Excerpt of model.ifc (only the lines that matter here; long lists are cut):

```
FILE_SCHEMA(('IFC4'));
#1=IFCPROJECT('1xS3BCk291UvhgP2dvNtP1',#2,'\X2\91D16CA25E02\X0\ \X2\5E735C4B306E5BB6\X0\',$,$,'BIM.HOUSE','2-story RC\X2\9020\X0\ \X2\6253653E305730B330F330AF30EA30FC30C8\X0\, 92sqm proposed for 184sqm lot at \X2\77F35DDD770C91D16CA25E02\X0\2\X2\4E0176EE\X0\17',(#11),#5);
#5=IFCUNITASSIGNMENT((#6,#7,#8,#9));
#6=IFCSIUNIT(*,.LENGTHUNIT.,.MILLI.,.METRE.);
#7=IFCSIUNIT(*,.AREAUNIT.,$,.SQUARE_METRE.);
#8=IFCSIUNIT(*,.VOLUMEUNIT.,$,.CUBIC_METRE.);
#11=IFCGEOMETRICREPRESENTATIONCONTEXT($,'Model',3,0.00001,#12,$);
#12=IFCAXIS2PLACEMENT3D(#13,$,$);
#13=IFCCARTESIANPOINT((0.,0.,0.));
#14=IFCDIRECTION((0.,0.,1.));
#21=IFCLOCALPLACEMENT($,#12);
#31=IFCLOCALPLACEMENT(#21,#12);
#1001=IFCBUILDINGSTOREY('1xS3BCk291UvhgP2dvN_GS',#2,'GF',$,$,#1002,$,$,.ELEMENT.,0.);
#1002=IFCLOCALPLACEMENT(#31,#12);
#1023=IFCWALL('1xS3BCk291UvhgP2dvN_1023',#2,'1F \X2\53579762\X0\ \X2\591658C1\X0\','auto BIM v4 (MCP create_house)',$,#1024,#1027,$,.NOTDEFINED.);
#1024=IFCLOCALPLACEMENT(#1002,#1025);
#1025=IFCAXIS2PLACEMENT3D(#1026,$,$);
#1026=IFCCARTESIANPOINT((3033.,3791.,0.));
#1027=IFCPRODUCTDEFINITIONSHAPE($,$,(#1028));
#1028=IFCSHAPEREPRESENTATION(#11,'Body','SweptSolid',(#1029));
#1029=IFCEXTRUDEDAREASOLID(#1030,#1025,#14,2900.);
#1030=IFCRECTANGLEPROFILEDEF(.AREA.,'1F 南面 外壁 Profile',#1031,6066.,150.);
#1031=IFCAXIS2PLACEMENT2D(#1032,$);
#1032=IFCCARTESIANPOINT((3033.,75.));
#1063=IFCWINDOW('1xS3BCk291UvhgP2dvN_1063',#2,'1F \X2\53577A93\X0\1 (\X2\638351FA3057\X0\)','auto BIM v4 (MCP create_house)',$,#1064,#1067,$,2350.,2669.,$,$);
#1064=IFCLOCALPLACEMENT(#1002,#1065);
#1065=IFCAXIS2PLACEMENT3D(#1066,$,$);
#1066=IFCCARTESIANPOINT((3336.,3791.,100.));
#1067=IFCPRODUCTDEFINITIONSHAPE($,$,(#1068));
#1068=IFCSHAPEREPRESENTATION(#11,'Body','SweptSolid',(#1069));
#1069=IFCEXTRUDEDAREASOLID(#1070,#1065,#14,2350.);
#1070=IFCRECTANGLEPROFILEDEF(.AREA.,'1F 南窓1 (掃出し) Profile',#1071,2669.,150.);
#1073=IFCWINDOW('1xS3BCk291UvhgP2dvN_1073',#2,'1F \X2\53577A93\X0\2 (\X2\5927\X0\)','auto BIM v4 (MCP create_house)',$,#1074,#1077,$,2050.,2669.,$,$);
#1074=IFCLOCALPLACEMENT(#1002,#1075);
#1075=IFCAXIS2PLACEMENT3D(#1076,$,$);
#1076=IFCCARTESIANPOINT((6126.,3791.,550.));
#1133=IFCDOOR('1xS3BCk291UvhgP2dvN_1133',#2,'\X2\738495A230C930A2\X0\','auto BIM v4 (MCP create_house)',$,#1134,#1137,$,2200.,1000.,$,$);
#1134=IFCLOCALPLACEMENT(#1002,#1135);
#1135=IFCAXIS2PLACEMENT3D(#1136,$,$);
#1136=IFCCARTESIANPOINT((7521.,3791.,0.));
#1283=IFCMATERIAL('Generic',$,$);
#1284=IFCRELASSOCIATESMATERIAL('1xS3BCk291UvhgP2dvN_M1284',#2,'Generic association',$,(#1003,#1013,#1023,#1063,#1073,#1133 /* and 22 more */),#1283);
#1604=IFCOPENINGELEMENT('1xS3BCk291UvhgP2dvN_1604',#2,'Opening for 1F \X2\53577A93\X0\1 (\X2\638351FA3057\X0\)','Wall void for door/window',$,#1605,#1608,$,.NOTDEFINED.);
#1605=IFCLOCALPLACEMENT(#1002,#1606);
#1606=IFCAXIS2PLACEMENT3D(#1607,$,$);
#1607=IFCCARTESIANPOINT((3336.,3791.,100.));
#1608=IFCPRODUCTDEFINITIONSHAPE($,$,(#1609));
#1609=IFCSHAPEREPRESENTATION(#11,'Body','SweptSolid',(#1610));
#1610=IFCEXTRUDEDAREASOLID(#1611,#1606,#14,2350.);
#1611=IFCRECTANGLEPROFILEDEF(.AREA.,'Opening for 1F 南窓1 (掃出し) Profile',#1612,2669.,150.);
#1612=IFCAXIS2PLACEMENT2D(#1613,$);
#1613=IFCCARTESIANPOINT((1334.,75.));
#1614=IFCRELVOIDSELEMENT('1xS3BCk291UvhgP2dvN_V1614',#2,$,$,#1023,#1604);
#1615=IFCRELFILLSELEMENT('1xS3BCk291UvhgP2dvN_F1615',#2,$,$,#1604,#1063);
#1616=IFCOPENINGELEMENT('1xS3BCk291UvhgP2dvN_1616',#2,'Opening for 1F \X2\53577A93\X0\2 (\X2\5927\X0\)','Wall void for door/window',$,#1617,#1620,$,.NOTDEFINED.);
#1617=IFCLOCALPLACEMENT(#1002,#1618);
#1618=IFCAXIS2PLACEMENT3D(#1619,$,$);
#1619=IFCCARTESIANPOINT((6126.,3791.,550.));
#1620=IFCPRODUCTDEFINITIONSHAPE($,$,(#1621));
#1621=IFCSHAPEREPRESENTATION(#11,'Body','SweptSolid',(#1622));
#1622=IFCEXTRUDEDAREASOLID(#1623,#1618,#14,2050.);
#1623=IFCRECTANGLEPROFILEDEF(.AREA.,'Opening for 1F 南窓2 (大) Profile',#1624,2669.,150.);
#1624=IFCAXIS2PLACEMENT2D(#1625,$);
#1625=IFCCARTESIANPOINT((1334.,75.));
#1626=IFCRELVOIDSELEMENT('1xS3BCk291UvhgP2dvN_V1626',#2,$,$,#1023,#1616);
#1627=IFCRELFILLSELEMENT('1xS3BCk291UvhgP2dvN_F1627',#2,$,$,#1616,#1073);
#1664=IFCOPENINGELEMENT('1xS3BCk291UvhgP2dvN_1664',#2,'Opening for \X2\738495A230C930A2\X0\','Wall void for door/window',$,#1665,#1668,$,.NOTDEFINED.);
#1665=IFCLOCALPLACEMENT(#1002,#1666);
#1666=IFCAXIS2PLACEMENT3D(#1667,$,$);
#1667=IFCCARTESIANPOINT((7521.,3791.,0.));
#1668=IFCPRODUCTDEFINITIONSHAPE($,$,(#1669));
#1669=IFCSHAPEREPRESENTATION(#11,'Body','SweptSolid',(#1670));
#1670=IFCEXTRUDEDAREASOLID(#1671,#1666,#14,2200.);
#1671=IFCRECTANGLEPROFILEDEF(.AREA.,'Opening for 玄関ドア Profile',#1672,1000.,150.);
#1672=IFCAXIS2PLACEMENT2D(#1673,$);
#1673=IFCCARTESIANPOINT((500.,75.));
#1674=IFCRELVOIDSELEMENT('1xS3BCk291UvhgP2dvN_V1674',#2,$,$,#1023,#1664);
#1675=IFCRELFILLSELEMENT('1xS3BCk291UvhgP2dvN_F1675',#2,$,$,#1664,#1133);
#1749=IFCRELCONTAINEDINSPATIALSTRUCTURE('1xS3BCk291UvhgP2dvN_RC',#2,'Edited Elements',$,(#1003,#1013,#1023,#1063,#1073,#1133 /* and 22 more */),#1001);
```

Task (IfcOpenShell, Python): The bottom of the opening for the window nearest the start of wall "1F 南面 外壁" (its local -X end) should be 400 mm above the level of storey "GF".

```python
import numpy as np
import ifcopenshell
import ifcopenshell.api.geometry
import ifcopenshell.geom
import ifcopenshell.util.element
import ifcopenshell.util.placement
import ifcopenshell.util.shape
import ifcopenshell.util.unit

model = ifcopenshell.open("model.ifc")
unit_scale = ifcopenshell.util.unit.calculate_unit_scale(model)

window = model.by_id(1063)
opening = window.FillsVoids[0].RelatingOpeningElement
storey = ifcopenshell.util.element.get_container(window, ifc_class="IfcBuildingStorey")
level = ifcopenshell.util.placement.get_local_placement(storey.ObjectPlacement)[2, 3]

# The opening's origin need not be at the sill, so measure its lowest point.
shape = ifcopenshell.geom.create_shape(ifcopenshell.geom.settings(), opening)
bottom = ifcopenshell.util.shape.get_shape_bottom_elevation(shape, shape.geometry) / unit_scale
dz = level + 400.0 - bottom

shift = np.array([0.0, 0.0, dz])
# The window is not placed relative to its opening, so move both.
for product in (opening, window):
    matrix = ifcopenshell.util.placement.get_local_placement(product.ObjectPlacement)
    matrix[:3, 3] += shift
    ifcopenshell.api.geometry.edit_object_placement(model, product=product, matrix=matrix, is_si=False)

print(f"moved by {dz * unit_scale:+.3f} m")

model.write("model_rev.ifc")
```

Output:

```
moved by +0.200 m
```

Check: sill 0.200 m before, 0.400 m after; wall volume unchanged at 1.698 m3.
